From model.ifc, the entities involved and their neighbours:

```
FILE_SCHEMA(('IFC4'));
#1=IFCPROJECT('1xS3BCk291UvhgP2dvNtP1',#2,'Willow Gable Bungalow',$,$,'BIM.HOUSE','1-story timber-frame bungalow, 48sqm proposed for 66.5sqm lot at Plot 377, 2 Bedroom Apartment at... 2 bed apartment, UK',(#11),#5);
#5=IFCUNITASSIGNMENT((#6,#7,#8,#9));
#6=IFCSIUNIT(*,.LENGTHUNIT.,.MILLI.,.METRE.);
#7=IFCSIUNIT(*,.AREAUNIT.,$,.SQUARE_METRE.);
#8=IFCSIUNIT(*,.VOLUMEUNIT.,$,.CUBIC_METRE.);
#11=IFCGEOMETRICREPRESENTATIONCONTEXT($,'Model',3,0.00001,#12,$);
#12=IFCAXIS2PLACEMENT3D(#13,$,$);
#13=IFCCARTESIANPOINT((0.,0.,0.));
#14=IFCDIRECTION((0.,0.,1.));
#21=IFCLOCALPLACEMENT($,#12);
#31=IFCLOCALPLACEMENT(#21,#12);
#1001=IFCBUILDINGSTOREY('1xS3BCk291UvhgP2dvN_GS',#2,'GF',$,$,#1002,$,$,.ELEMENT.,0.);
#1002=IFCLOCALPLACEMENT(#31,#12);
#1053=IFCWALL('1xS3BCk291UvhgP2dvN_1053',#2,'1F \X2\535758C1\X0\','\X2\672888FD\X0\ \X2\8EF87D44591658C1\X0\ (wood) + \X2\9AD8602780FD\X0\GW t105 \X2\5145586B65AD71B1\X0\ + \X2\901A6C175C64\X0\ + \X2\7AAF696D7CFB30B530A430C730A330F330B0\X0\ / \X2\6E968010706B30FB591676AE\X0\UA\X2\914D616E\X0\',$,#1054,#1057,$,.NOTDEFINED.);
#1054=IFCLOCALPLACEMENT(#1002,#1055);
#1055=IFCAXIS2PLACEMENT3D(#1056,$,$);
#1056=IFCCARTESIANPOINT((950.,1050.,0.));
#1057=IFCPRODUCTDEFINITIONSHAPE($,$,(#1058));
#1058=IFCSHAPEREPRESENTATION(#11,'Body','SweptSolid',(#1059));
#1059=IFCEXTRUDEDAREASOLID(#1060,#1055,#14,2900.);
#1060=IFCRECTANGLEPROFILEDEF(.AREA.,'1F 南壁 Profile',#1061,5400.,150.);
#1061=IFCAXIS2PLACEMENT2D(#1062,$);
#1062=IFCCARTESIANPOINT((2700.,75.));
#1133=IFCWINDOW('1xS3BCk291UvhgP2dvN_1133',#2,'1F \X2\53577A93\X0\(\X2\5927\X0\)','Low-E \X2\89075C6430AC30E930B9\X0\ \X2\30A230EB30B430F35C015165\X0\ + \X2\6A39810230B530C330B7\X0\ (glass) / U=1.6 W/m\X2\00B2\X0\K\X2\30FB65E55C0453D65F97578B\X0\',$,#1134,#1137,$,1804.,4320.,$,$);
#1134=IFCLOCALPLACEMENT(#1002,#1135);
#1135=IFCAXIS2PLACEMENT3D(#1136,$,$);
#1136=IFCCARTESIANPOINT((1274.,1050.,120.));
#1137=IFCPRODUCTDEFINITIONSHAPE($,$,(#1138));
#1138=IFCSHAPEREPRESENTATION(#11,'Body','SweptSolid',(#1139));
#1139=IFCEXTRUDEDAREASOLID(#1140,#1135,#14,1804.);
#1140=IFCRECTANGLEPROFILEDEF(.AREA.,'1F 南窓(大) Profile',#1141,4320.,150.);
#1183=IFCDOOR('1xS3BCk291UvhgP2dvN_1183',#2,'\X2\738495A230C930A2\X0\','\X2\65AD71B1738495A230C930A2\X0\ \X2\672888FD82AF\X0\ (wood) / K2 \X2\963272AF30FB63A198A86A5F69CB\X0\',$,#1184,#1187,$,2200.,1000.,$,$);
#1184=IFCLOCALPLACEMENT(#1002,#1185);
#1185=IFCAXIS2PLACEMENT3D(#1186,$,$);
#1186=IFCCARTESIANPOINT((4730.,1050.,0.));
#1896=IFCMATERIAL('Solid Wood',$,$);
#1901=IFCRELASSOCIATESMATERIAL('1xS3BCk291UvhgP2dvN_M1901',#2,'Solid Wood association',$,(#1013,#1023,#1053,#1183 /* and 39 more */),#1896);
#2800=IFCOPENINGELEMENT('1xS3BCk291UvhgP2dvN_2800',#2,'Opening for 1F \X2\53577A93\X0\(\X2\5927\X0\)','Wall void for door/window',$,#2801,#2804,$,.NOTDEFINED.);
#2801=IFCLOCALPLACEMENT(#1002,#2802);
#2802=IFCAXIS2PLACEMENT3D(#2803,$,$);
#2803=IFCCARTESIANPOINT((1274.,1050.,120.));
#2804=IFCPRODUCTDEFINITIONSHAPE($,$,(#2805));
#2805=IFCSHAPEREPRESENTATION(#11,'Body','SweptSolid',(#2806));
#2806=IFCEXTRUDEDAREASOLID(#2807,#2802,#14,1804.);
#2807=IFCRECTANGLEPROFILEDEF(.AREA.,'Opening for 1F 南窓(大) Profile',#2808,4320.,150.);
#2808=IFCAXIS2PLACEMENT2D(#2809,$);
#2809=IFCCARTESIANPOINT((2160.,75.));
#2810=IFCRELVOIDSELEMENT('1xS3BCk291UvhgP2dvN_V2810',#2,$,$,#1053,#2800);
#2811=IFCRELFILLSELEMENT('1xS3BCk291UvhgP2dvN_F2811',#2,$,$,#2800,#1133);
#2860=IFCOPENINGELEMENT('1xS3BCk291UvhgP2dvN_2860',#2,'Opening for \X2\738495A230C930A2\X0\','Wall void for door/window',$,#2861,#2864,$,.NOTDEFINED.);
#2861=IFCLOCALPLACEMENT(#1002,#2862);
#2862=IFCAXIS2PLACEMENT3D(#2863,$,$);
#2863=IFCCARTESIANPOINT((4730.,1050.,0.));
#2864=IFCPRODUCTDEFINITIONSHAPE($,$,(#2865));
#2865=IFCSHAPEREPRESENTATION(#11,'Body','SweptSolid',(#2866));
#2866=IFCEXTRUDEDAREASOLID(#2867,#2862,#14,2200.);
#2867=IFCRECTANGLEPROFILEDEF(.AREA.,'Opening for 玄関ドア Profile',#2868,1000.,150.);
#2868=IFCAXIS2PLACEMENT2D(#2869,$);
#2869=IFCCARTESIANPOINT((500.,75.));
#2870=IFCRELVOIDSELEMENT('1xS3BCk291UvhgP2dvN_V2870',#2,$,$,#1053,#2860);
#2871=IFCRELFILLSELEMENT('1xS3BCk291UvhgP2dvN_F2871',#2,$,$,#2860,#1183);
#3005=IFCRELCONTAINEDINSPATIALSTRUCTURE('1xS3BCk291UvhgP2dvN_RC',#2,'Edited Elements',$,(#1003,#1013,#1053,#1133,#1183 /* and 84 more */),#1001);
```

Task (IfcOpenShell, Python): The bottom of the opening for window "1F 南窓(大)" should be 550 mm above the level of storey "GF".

```python
import numpy as np
import ifcopenshell
import ifcopenshell.api.geometry
import ifcopenshell.geom
import ifcopenshell.util.element
import ifcopenshell.util.placement
import ifcopenshell.util.shape
import ifcopenshell.util.unit

model = ifcopenshell.open("model.ifc")
unit_scale = ifcopenshell.util.unit.calculate_unit_scale(model)

window = model.by_guid("1xS3BCk291UvhgP2dvN_1133")
opening = window.FillsVoids[0].RelatingOpeningElement
storey = ifcopenshell.util.element.get_container(window, ifc_class="IfcBuildingStorey")
level = ifcopenshell.util.placement.get_local_placement(storey.ObjectPlacement)[2, 3]

# The opening's origin need not be at the sill, so measure its lowest point.
shape = ifcopenshell.geom.create_shape(ifcopenshell.geom.settings(), opening)
bottom = ifcopenshell.util.shape.get_shape_bottom_elevation(shape, shape.geometry) / unit_scale
dz = level + 550.0 - bottom

shift = np.array([0.0, 0.0, dz])
# The window is not placed relative to its opening, so move both.
for product in (opening, window):
    matrix = ifcopenshell.util.placement.get_local_placement(product.ObjectPlacement)
    matrix[:3, 3] += shift
    ifcopenshell.api.geometry.edit_object_placement(model, product=product, matrix=matrix, is_si=False)

print(f"moved by {dz * unit_scale:+.3f} m")

model.write("model_updated.ifc")
```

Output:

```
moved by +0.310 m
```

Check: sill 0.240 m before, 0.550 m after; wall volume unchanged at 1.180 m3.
